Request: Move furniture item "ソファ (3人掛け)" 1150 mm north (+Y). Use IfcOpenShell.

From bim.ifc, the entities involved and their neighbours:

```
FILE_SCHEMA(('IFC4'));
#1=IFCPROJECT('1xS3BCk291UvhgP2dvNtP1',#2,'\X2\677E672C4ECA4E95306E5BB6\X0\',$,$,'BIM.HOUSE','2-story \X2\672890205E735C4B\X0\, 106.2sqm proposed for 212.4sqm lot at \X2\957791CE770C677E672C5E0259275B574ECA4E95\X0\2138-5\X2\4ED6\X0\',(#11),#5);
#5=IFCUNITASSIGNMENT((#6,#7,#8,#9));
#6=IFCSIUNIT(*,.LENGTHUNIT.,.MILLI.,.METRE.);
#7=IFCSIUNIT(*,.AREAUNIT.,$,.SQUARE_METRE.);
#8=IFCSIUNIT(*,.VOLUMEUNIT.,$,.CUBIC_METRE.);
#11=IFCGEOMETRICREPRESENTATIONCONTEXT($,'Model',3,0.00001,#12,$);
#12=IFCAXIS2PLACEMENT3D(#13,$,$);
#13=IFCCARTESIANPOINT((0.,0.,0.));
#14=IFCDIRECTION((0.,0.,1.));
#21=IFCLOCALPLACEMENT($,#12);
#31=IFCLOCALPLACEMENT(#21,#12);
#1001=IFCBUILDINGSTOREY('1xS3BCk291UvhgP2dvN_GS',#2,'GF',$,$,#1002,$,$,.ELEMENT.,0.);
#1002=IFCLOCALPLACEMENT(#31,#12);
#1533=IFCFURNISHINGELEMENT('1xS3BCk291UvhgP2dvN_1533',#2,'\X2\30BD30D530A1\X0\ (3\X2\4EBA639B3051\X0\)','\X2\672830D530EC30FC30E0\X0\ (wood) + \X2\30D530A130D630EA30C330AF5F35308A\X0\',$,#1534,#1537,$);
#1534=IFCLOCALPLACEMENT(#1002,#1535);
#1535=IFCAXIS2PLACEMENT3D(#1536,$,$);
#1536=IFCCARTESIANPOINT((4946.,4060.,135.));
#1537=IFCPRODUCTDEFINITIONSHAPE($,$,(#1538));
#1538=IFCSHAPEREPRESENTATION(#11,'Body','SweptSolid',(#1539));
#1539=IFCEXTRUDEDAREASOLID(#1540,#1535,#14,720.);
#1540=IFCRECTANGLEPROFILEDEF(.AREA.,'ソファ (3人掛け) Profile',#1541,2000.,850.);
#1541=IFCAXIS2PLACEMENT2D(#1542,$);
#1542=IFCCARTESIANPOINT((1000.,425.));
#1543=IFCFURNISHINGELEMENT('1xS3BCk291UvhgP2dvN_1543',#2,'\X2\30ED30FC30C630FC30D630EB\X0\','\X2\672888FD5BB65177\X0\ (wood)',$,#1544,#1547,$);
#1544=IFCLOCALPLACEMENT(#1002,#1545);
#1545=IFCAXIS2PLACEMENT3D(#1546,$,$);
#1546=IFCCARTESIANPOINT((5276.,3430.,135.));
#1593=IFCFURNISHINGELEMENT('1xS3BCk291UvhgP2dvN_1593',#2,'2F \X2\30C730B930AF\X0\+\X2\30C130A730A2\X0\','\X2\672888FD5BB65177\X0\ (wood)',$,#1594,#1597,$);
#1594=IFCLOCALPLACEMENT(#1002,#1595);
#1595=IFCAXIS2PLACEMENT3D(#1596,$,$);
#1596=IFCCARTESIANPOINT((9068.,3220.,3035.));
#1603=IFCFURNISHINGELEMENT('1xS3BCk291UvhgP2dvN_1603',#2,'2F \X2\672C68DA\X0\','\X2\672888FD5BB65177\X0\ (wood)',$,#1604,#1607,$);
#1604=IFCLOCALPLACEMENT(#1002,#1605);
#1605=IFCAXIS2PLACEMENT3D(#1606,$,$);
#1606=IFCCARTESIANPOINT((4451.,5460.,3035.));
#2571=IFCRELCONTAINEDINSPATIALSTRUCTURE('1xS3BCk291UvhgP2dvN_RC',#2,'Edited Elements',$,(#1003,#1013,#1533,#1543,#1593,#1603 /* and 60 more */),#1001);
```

```python
import ifcopenshell
import ifcopenshell.api.geometry
import ifcopenshell.util.placement
import ifcopenshell.util.unit

model = ifcopenshell.open("bim.ifc")
unit_scale = ifcopenshell.util.unit.calculate_unit_scale(model)

item = model.by_guid("1xS3BCk291UvhgP2dvN_1533")
matrix = ifcopenshell.util.placement.get_local_placement(item.ObjectPlacement)
matrix[1, 3] += 1.15 / unit_scale
ifcopenshell.api.geometry.edit_object_placement(model, product=item, matrix=matrix, is_si=False)

print(ifcopenshell.util.placement.get_local_placement(item.ObjectPlacement).round(3) + 0.0)

model.write("bim-out.ifc")
```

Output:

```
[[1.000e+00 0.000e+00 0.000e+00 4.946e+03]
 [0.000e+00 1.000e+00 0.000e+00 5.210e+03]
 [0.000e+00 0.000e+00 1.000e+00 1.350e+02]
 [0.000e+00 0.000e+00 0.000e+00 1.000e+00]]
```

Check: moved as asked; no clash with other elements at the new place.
